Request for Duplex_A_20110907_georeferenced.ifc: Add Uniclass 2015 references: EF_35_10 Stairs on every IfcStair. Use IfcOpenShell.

First a look at what the model holds.

```python
import ifcopenshell

model = ifcopenshell.open("Duplex_A_20110907_georeferenced.ifc")
print(model.schema)
print("classifications:", [c.Name for c in model.by_type("IfcClassification")])
for ifc_class in ("IfcDoor", "IfcRoof", "IfcStair", "IfcWall", "IfcWindow"):
    print(ifc_class, len(model.by_type(ifc_class)))
```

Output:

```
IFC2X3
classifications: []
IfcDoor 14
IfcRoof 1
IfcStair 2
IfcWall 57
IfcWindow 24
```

```python
import ifcopenshell
import ifcopenshell.api.classification

model = ifcopenshell.open("Duplex_A_20110907_georeferenced.ifc")

# IFC2X3 requires Source and Edition and has no link from the project to the system.
system = model.create_entity("IfcClassification", Source="NBS", Edition="2015", Name="Uniclass 2015")

codes = {
    "IfcStair": ("EF_35_10", "Stairs"),
}
for ifc_class, (code, name) in codes.items():
    products = model.by_type(ifc_class)
    ifcopenshell.api.classification.add_reference(
        model, products=products, classification=system, identification=code, name=name
    )
    print(code, len(products))

model.write("Duplex_A_20110907_georeferenced_v2.ifc")
```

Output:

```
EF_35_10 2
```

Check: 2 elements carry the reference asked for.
